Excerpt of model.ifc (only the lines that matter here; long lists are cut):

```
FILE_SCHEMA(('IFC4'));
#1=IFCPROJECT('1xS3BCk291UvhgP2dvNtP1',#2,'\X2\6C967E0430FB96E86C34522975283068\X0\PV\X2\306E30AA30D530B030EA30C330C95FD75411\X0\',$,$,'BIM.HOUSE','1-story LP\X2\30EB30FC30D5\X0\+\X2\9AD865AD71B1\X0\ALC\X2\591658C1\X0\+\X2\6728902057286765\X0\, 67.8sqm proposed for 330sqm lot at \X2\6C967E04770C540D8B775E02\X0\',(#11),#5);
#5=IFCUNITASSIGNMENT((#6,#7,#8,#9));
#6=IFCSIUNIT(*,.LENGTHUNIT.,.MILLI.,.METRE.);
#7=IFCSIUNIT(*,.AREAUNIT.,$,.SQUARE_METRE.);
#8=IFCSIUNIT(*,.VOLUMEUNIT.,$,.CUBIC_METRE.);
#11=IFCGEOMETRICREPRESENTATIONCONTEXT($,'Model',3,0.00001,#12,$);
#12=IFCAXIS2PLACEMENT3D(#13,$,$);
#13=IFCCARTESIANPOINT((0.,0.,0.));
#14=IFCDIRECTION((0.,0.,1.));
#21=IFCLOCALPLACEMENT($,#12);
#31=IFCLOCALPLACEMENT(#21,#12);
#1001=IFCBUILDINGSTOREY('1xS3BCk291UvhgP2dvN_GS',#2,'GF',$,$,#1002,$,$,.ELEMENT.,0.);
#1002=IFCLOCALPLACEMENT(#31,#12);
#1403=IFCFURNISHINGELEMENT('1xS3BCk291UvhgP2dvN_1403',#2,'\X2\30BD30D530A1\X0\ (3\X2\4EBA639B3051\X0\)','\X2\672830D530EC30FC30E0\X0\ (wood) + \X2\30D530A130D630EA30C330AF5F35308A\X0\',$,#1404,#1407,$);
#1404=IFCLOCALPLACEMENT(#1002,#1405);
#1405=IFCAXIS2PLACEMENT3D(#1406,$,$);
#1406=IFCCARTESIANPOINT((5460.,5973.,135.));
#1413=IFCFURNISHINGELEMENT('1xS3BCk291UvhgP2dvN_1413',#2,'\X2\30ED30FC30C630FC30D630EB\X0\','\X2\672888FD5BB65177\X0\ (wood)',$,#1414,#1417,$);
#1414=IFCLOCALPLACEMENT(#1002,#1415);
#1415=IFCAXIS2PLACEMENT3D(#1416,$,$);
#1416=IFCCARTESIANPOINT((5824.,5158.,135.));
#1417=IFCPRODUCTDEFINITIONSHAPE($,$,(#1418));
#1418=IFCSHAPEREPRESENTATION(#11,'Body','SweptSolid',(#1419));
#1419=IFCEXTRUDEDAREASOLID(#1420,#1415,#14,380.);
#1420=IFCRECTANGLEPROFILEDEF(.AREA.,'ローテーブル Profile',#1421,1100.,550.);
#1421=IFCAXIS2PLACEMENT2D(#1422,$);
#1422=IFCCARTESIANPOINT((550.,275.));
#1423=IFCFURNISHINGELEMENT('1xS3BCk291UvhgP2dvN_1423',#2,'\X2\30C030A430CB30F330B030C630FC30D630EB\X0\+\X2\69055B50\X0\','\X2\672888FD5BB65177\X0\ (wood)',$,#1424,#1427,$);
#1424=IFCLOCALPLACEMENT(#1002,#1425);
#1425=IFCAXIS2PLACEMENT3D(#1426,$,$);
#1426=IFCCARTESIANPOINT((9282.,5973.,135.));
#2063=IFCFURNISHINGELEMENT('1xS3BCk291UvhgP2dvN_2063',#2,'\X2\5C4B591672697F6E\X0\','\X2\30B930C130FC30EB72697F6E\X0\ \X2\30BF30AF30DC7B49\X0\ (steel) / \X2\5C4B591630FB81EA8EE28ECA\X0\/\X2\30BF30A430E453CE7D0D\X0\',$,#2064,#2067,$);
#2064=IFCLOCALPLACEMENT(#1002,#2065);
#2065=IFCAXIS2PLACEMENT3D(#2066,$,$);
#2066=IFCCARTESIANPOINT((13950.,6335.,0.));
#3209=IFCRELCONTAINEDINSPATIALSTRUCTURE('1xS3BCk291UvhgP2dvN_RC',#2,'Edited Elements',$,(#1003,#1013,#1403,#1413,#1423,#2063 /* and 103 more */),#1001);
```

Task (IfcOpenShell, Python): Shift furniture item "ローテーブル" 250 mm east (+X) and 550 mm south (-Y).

```python
import ifcopenshell
import ifcopenshell.api.geometry
import ifcopenshell.util.placement

model = ifcopenshell.open("model.ifc")

item = model.by_guid("1xS3BCk291UvhgP2dvN_1413")
matrix = ifcopenshell.util.placement.get_local_placement(item.ObjectPlacement)
matrix[0, 3] += 250.0
matrix[1, 3] -= 550.0
ifcopenshell.api.geometry.edit_object_placement(model, product=item, matrix=matrix, is_si=False)

print(ifcopenshell.util.placement.get_local_placement(item.ObjectPlacement).round(3) + 0.0)

model.write("model_rev.ifc")
```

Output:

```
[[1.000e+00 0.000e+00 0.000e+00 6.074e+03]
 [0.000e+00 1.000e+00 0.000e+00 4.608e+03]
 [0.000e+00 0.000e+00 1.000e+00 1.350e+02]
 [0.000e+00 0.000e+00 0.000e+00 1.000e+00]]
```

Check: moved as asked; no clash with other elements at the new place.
